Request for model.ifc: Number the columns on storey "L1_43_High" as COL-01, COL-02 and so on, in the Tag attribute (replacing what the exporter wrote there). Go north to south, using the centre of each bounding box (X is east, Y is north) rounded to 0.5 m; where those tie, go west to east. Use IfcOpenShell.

First a look at what the model holds.

```python
import ifcopenshell
import ifcopenshell.util.element
import ifcopenshell.util.placement

model = ifcopenshell.open("model.ifc")
print(model.schema)
storey = next(s for s in model.by_type("IfcBuildingStorey") if s.Name == "L1_43_High")
columns = [e for e in ifcopenshell.util.element.get_decomposition(storey) if e.is_a("IfcColumn")]
for e in sorted(columns, key=lambda e: e.id()):
    origin = ifcopenshell.util.placement.get_local_placement(e.ObjectPlacement)[:3, 3]
    print(e.id(), e.Tag, e.Name, origin.round(2) + 0.0, sep=" | ")
```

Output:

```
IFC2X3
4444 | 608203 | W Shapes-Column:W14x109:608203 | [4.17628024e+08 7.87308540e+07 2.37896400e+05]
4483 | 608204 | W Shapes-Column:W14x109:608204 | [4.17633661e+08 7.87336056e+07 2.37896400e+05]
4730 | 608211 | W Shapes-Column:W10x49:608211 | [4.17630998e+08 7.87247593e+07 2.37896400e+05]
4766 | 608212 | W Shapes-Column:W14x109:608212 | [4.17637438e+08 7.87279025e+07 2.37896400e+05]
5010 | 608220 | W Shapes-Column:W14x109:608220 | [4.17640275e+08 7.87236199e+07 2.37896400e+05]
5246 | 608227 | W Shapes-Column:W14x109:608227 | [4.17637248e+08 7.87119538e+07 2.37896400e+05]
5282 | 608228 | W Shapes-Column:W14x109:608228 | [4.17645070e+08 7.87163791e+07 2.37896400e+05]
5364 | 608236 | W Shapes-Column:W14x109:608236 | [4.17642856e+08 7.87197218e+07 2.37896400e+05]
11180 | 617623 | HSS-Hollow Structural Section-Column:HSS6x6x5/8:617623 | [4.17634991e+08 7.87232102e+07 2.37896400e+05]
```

```python
import ifcopenshell
import ifcopenshell.geom
import ifcopenshell.util.element
import ifcopenshell.util.shape

model = ifcopenshell.open("model.ifc")
settings = ifcopenshell.geom.settings()
settings.set("use-world-coords", True)


def centre(element):
    shape = ifcopenshell.geom.create_shape(settings, element)
    return ifcopenshell.util.shape.get_bbox_centroid(shape.geometry)


storey = next(s for s in model.by_type("IfcBuildingStorey") if s.Name == "L1_43_High")
columns = [e for e in ifcopenshell.util.element.get_decomposition(storey) if e.is_a("IfcColumn")]

# Insertion points can sit at a corner or the storey origin, so sort by the geometry (in metres).
centres = {e: centre(e) for e in columns}
columns.sort(key=lambda e: (-round(centres[e][1] / 0.5), centres[e][0]))

for i, e in enumerate(columns, start=1):
    number = f"COL-{i:02d}"
    e.Tag = number
    print(e.id(), number)

model.write("model_updated.ifc")
```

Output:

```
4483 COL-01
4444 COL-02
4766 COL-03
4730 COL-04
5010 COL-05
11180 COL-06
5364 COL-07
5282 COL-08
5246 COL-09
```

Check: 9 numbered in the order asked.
